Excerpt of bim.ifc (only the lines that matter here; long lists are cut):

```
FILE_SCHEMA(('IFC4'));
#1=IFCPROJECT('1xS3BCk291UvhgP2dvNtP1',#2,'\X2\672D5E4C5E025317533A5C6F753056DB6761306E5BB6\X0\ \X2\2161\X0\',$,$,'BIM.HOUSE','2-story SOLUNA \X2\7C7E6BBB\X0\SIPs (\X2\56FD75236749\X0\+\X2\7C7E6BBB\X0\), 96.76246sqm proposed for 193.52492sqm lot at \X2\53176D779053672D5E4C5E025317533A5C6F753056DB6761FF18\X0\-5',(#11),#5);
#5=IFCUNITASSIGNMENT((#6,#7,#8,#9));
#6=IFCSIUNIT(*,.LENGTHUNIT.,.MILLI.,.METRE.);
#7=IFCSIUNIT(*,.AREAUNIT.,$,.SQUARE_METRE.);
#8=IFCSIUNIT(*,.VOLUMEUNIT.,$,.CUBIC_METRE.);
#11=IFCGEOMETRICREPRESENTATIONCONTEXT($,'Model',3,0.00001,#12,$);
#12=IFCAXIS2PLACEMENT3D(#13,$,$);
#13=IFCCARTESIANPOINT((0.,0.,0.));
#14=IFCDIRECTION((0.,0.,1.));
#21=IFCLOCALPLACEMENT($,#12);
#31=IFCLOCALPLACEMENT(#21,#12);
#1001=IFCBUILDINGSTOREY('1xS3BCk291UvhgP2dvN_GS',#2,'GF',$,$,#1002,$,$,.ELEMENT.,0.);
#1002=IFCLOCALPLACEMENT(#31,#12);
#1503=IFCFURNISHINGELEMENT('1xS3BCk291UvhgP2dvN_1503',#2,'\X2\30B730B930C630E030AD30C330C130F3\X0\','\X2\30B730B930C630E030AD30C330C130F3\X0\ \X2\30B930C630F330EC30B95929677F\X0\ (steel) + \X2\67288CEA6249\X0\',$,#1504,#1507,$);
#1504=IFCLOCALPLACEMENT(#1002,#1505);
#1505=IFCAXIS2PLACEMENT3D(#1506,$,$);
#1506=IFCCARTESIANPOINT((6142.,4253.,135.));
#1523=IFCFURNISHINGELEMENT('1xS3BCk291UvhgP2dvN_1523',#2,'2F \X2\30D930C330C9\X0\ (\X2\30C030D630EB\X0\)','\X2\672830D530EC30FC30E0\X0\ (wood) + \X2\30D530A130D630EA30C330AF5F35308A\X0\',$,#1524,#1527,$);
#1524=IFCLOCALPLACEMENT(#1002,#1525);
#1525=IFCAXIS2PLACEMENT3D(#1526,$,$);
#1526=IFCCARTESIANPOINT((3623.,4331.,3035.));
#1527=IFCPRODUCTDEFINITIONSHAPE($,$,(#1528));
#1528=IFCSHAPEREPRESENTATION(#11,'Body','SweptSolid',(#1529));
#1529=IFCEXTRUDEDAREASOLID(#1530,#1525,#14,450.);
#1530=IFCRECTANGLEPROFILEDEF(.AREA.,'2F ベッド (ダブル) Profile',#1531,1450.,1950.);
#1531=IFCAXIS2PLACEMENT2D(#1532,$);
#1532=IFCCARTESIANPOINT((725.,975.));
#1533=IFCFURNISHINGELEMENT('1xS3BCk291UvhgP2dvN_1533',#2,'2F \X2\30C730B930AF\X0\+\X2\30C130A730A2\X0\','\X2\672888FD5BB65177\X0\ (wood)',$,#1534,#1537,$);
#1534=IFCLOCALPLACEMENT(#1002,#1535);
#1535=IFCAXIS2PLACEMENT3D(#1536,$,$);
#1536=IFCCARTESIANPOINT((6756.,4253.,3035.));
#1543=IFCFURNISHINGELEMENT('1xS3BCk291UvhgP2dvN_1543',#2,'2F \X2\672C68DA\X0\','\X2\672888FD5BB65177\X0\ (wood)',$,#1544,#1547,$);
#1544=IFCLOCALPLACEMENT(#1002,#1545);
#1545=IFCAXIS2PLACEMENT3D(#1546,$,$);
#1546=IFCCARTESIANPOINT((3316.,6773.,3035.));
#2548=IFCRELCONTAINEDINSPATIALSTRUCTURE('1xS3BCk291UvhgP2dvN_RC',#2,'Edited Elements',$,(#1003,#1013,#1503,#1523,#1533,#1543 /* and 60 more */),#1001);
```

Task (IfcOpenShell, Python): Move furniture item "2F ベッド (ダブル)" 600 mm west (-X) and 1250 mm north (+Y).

```python
import ifcopenshell
import ifcopenshell.api.geometry
import ifcopenshell.util.placement

model = ifcopenshell.open("bim.ifc")

item = model.by_guid("1xS3BCk291UvhgP2dvN_1523")
matrix = ifcopenshell.util.placement.get_local_placement(item.ObjectPlacement)
matrix[0, 3] -= 600.0
matrix[1, 3] += 1250.0
ifcopenshell.api.geometry.edit_object_placement(model, product=item, matrix=matrix, is_si=False)

print(ifcopenshell.util.placement.get_local_placement(item.ObjectPlacement).round(3) + 0.0)

model.write("bim-out.ifc")
```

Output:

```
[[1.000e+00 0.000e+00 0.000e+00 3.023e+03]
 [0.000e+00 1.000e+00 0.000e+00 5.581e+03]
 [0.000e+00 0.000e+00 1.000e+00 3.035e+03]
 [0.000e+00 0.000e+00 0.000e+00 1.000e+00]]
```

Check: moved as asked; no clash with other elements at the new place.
